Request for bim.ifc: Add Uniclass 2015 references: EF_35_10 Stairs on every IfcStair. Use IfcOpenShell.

First a look at what the model holds.

```python
import ifcopenshell

model = ifcopenshell.open("bim.ifc")
print(model.schema)
print("classifications:", [c.Name for c in model.by_type("IfcClassification")])
for ifc_class in ("IfcDoor", "IfcRoof", "IfcStair", "IfcWall", "IfcWindow"):
    print(ifc_class, len(model.by_type(ifc_class)))
```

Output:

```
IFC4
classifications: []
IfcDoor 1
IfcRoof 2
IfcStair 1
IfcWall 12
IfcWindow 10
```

```python
import ifcopenshell
import ifcopenshell.api.classification

model = ifcopenshell.open("bim.ifc")

system = ifcopenshell.api.classification.add_classification(model, classification="Uniclass 2015")

codes = {
    "IfcStair": ("EF_35_10", "Stairs"),
}
for ifc_class, (code, name) in codes.items():
    products = model.by_type(ifc_class)
    ifcopenshell.api.classification.add_reference(
        model, products=products, classification=system, identification=code, name=name
    )
    print(code, len(products))

model.write("bim-out.ifc")
```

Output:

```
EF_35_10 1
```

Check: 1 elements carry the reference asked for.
